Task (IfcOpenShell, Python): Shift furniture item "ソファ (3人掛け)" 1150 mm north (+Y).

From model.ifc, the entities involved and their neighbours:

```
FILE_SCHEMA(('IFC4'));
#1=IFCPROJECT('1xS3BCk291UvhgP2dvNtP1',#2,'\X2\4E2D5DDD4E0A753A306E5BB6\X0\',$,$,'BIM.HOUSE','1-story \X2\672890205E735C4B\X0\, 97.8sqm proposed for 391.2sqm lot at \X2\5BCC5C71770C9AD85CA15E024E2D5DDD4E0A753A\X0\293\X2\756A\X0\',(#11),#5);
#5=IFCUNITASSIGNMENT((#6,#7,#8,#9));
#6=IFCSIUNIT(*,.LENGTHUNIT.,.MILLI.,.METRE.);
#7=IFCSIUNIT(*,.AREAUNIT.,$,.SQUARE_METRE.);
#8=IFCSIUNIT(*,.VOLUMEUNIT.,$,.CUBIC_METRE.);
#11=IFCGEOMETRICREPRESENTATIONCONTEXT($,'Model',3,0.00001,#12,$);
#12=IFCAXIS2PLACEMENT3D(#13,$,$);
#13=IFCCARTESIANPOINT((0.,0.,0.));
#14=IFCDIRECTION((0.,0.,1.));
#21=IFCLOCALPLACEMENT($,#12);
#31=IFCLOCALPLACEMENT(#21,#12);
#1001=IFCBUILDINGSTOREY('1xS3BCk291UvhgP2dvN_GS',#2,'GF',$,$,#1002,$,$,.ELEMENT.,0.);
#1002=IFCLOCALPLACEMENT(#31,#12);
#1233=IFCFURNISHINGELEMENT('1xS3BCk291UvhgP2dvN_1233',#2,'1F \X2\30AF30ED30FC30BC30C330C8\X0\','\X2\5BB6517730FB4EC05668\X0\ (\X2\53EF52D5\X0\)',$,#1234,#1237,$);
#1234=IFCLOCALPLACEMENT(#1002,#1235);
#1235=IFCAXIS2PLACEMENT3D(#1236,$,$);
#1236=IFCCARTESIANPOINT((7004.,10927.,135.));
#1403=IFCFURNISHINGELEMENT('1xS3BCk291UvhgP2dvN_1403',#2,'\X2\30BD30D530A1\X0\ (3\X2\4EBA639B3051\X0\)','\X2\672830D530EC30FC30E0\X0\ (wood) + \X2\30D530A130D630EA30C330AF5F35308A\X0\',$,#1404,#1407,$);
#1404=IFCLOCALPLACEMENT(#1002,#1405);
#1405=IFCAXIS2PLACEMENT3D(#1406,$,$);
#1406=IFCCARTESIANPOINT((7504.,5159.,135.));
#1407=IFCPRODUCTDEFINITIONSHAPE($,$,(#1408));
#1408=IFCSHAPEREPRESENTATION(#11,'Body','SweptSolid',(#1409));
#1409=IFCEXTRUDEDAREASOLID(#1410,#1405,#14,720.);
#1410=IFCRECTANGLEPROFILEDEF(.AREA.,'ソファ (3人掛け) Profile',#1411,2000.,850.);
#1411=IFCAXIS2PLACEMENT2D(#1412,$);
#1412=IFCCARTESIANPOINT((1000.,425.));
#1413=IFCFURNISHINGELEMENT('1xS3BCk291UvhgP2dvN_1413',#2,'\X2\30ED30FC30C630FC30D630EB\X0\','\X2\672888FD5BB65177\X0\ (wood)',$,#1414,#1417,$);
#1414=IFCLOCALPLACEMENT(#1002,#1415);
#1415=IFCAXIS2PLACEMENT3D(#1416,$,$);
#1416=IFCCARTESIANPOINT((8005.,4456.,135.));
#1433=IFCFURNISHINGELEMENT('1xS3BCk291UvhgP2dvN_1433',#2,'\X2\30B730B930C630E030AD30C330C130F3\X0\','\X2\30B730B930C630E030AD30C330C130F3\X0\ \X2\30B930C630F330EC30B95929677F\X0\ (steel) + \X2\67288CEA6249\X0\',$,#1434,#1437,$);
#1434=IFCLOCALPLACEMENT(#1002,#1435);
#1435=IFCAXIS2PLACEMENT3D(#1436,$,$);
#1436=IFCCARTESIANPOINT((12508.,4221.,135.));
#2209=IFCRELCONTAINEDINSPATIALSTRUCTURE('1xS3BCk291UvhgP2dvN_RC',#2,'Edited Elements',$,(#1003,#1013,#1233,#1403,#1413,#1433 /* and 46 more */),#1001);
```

```python
import ifcopenshell
import ifcopenshell.api.geometry
import ifcopenshell.util.placement

model = ifcopenshell.open("model.ifc")

item = model.by_guid("1xS3BCk291UvhgP2dvN_1403")
matrix = ifcopenshell.util.placement.get_local_placement(item.ObjectPlacement)
matrix[1, 3] += 1150.0
ifcopenshell.api.geometry.edit_object_placement(model, product=item, matrix=matrix, is_si=False)

print(ifcopenshell.util.placement.get_local_placement(item.ObjectPlacement).round(3) + 0.0)

model.write("model_updated.ifc")
```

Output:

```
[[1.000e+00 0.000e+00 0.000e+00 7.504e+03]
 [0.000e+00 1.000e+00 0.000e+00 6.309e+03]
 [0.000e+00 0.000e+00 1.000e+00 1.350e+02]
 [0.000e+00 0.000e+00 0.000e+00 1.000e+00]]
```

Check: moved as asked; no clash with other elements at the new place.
